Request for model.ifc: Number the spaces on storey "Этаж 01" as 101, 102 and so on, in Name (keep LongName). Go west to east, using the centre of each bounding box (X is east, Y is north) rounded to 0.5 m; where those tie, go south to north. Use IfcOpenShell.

First a look at what the model holds.

```python
import ifcopenshell
import ifcopenshell.util.element
import ifcopenshell.util.placement

model = ifcopenshell.open("model.ifc")
print(model.schema)
storey = next(s for s in model.by_type("IfcBuildingStorey") if s.Name == "Этаж 01")
spaces = [e for e in ifcopenshell.util.element.get_decomposition(storey) if e.is_a("IfcSpace")]
for e in sorted(spaces, key=lambda e: e.id()):
    origin = ifcopenshell.util.placement.get_local_placement(e.ObjectPlacement)[:3, 3]
    print(e.id(), e.Name, e.LongName, origin.round(2) + 0.0, sep=" | ")
```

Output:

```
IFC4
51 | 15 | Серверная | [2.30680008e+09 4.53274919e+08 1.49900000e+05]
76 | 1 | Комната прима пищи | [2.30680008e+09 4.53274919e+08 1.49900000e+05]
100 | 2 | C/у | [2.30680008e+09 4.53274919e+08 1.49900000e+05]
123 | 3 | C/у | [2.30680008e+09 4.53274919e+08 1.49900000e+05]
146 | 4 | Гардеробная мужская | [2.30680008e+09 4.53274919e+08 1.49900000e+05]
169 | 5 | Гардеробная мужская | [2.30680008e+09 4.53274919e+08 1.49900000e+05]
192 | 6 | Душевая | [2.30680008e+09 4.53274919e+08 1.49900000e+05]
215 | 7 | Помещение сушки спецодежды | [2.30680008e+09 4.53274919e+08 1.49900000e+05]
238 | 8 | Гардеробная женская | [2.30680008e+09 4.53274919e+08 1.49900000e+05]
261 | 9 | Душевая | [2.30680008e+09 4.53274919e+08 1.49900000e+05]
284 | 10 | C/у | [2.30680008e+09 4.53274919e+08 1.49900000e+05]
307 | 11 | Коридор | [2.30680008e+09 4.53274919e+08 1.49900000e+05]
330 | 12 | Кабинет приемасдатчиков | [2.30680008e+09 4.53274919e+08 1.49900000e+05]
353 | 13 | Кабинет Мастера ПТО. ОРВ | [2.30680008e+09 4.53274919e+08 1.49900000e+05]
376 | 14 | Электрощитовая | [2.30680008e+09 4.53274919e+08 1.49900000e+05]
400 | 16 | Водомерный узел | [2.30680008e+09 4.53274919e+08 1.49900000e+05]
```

```python
import ifcopenshell
import ifcopenshell.geom
import ifcopenshell.util.element
import ifcopenshell.util.shape

model = ifcopenshell.open("model.ifc")
settings = ifcopenshell.geom.settings()
settings.set("use-world-coords", True)


def centre(element):
    shape = ifcopenshell.geom.create_shape(settings, element)
    return ifcopenshell.util.shape.get_bbox_centroid(shape.geometry)


storey = next(s for s in model.by_type("IfcBuildingStorey") if s.Name == "Этаж 01")
spaces = [e for e in ifcopenshell.util.element.get_decomposition(storey) if e.is_a("IfcSpace")]

# Insertion points can sit at a corner or the storey origin, so sort by the geometry (in metres).
centres = {e: centre(e) for e in spaces}
spaces.sort(key=lambda e: (round(centres[e][0] / 0.5), centres[e][1]))

for i, e in enumerate(spaces, start=1):
    number = f"1{i:02d}"
    e.Name = number
    print(e.id(), number)

model.write("model_updated.ifc")
```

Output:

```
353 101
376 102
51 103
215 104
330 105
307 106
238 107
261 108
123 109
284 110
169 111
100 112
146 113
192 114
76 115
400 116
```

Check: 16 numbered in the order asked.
